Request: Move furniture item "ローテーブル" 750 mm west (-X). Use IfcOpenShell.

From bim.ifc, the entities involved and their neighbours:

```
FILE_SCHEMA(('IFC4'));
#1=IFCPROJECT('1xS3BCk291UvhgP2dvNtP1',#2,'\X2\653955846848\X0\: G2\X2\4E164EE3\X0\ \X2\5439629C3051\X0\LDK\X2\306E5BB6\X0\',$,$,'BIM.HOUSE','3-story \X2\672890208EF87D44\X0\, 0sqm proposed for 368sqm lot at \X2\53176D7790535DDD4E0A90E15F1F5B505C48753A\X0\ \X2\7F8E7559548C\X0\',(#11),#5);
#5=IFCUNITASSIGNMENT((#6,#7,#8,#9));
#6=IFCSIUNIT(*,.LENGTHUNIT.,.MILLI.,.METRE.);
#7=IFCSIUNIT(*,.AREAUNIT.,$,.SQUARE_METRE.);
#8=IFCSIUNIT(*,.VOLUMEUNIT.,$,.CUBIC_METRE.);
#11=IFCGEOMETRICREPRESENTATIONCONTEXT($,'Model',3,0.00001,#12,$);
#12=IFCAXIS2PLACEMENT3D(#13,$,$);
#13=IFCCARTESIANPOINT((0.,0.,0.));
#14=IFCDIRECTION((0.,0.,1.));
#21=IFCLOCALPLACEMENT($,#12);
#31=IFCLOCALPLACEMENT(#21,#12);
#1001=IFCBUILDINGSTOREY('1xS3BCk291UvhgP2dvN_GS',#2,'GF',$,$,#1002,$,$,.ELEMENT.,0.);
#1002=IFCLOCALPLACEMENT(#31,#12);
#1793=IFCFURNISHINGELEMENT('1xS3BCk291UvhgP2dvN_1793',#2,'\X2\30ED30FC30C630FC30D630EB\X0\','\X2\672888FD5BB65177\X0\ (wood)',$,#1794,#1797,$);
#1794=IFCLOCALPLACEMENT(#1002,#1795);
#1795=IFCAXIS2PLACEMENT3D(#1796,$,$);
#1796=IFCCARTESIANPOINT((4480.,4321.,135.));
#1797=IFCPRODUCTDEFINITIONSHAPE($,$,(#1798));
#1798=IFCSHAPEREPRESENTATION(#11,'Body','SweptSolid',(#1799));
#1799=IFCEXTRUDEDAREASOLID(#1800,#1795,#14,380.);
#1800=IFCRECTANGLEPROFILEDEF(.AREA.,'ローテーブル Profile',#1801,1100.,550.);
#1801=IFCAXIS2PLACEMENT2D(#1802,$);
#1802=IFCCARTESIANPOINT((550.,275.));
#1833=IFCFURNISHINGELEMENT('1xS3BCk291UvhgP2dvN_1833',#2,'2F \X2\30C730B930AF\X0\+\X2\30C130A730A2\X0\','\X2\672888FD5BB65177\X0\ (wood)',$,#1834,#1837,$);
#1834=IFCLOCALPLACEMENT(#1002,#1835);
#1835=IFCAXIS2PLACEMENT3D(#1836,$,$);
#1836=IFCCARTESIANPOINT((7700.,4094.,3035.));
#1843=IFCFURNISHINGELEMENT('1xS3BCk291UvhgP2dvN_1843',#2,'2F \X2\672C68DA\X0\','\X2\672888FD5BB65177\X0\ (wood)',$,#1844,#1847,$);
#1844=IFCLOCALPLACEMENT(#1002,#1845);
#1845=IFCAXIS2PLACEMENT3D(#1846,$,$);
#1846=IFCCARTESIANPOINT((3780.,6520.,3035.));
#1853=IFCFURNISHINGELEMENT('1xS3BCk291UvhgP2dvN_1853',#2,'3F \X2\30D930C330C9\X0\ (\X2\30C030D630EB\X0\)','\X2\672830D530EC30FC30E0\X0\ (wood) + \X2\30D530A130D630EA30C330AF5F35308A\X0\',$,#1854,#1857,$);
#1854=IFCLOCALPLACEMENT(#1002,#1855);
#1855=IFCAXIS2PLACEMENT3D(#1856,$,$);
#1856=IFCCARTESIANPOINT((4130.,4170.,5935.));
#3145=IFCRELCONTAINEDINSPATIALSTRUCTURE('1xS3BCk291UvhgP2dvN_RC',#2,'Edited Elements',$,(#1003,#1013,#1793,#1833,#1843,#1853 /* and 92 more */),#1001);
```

```python
import ifcopenshell
import ifcopenshell.api.geometry
import ifcopenshell.util.placement
import ifcopenshell.util.unit

model = ifcopenshell.open("bim.ifc")
unit_scale = ifcopenshell.util.unit.calculate_unit_scale(model)

item = model.by_id(1793)
matrix = ifcopenshell.util.placement.get_local_placement(item.ObjectPlacement)
matrix[0, 3] -= 0.75 / unit_scale
ifcopenshell.api.geometry.edit_object_placement(model, product=item, matrix=matrix, is_si=False)

print(ifcopenshell.util.placement.get_local_placement(item.ObjectPlacement).round(3) + 0.0)

model.write("bim_updated.ifc")
```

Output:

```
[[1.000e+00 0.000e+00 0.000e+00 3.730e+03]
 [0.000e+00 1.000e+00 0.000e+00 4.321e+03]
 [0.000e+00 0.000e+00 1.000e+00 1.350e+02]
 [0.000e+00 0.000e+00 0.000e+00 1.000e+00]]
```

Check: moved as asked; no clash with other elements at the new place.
